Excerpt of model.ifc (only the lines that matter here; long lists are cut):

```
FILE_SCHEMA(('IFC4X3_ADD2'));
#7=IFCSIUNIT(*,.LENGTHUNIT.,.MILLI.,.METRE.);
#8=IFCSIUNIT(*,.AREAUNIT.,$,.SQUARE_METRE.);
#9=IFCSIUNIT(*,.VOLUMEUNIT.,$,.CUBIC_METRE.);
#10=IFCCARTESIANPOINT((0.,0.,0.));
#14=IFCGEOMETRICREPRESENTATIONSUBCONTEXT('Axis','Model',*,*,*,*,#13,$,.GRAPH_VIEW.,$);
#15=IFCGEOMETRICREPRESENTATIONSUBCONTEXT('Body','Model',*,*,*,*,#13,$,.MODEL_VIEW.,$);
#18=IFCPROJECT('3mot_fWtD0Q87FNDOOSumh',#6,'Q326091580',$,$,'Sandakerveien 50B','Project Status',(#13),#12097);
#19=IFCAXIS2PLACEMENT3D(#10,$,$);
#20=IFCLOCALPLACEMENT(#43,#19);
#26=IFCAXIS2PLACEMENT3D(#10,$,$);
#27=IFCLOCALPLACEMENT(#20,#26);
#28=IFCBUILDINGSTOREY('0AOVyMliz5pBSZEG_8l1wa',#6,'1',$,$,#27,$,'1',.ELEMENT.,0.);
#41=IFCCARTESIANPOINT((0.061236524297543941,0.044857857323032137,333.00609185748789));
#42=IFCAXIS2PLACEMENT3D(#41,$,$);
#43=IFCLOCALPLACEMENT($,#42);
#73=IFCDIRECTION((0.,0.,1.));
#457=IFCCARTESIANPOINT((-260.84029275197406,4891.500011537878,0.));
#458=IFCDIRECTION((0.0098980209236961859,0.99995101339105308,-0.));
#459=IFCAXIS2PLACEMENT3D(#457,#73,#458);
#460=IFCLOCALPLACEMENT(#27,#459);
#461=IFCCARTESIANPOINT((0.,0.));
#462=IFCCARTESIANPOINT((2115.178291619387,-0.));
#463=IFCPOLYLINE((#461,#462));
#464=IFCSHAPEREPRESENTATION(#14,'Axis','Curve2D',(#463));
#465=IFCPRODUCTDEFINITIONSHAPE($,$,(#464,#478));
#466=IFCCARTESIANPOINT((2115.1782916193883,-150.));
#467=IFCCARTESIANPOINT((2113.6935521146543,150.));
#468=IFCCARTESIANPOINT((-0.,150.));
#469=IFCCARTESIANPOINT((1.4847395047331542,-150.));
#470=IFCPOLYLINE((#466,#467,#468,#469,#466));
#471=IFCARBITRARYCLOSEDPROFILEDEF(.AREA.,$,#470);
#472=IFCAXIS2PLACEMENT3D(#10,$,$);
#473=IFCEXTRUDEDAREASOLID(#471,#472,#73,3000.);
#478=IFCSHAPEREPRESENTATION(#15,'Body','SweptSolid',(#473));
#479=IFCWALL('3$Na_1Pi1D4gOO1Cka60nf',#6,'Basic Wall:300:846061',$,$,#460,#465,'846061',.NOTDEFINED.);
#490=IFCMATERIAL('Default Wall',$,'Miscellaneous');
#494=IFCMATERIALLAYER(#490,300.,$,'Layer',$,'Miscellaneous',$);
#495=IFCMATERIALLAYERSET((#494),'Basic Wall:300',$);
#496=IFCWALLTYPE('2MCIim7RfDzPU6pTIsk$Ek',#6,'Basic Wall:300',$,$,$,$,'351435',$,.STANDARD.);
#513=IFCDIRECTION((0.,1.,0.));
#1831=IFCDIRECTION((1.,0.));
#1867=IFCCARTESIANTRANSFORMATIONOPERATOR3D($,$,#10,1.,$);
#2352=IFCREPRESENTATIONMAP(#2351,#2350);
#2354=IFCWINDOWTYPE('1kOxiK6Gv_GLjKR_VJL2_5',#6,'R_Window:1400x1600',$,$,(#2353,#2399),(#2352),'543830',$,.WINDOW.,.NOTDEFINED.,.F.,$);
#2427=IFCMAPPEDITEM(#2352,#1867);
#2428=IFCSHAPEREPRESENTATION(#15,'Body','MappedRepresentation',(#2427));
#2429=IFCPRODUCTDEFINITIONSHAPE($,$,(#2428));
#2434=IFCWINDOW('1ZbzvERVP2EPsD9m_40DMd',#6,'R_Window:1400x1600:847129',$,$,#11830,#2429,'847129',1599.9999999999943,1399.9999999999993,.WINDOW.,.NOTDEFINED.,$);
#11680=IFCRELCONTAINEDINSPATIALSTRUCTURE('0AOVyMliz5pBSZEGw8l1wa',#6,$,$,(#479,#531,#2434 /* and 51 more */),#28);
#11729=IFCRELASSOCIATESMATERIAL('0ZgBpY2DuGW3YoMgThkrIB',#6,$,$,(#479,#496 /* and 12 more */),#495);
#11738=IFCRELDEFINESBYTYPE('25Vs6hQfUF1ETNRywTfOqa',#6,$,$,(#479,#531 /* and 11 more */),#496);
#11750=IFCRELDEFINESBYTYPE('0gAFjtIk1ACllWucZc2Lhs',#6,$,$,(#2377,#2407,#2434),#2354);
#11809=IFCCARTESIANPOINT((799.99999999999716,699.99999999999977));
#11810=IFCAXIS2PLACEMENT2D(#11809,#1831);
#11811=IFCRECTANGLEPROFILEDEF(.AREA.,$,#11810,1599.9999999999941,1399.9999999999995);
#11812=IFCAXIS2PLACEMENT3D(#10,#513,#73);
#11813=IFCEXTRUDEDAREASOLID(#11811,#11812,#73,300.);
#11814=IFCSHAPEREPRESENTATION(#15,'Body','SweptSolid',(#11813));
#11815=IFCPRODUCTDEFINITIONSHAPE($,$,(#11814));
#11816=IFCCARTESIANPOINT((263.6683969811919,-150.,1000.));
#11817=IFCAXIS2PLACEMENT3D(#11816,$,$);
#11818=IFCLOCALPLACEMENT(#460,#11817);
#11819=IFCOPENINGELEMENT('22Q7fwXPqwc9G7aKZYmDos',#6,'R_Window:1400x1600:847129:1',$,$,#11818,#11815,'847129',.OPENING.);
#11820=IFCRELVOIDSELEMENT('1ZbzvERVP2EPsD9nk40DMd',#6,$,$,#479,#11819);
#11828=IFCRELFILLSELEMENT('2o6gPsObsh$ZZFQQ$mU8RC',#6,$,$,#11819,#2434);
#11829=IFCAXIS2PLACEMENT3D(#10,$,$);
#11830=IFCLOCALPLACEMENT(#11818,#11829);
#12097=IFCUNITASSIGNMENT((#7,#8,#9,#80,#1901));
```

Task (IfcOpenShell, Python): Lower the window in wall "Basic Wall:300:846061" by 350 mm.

```python
import numpy as np
import ifcopenshell
import ifcopenshell.api.geometry
import ifcopenshell.util.placement
import ifcopenshell.util.unit

model = ifcopenshell.open("model.ifc")
unit_scale = ifcopenshell.util.unit.calculate_unit_scale(model)

window = model.by_guid("1ZbzvERVP2EPsD9m_40DMd")
opening = window.FillsVoids[0].RelatingOpeningElement
dz = -350.0

shift = np.array([0.0, 0.0, dz])
# The window is placed relative to its opening, so it follows when the opening moves.
matrix = ifcopenshell.util.placement.get_local_placement(opening.ObjectPlacement)
matrix[:3, 3] += shift
ifcopenshell.api.geometry.edit_object_placement(
    model, product=opening, matrix=matrix, is_si=False, should_transform_children=True
)

print(f"moved by {dz * unit_scale:+.3f} m")

model.write("model_v2.ifc")
```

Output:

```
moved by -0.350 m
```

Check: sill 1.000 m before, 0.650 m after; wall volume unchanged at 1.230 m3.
